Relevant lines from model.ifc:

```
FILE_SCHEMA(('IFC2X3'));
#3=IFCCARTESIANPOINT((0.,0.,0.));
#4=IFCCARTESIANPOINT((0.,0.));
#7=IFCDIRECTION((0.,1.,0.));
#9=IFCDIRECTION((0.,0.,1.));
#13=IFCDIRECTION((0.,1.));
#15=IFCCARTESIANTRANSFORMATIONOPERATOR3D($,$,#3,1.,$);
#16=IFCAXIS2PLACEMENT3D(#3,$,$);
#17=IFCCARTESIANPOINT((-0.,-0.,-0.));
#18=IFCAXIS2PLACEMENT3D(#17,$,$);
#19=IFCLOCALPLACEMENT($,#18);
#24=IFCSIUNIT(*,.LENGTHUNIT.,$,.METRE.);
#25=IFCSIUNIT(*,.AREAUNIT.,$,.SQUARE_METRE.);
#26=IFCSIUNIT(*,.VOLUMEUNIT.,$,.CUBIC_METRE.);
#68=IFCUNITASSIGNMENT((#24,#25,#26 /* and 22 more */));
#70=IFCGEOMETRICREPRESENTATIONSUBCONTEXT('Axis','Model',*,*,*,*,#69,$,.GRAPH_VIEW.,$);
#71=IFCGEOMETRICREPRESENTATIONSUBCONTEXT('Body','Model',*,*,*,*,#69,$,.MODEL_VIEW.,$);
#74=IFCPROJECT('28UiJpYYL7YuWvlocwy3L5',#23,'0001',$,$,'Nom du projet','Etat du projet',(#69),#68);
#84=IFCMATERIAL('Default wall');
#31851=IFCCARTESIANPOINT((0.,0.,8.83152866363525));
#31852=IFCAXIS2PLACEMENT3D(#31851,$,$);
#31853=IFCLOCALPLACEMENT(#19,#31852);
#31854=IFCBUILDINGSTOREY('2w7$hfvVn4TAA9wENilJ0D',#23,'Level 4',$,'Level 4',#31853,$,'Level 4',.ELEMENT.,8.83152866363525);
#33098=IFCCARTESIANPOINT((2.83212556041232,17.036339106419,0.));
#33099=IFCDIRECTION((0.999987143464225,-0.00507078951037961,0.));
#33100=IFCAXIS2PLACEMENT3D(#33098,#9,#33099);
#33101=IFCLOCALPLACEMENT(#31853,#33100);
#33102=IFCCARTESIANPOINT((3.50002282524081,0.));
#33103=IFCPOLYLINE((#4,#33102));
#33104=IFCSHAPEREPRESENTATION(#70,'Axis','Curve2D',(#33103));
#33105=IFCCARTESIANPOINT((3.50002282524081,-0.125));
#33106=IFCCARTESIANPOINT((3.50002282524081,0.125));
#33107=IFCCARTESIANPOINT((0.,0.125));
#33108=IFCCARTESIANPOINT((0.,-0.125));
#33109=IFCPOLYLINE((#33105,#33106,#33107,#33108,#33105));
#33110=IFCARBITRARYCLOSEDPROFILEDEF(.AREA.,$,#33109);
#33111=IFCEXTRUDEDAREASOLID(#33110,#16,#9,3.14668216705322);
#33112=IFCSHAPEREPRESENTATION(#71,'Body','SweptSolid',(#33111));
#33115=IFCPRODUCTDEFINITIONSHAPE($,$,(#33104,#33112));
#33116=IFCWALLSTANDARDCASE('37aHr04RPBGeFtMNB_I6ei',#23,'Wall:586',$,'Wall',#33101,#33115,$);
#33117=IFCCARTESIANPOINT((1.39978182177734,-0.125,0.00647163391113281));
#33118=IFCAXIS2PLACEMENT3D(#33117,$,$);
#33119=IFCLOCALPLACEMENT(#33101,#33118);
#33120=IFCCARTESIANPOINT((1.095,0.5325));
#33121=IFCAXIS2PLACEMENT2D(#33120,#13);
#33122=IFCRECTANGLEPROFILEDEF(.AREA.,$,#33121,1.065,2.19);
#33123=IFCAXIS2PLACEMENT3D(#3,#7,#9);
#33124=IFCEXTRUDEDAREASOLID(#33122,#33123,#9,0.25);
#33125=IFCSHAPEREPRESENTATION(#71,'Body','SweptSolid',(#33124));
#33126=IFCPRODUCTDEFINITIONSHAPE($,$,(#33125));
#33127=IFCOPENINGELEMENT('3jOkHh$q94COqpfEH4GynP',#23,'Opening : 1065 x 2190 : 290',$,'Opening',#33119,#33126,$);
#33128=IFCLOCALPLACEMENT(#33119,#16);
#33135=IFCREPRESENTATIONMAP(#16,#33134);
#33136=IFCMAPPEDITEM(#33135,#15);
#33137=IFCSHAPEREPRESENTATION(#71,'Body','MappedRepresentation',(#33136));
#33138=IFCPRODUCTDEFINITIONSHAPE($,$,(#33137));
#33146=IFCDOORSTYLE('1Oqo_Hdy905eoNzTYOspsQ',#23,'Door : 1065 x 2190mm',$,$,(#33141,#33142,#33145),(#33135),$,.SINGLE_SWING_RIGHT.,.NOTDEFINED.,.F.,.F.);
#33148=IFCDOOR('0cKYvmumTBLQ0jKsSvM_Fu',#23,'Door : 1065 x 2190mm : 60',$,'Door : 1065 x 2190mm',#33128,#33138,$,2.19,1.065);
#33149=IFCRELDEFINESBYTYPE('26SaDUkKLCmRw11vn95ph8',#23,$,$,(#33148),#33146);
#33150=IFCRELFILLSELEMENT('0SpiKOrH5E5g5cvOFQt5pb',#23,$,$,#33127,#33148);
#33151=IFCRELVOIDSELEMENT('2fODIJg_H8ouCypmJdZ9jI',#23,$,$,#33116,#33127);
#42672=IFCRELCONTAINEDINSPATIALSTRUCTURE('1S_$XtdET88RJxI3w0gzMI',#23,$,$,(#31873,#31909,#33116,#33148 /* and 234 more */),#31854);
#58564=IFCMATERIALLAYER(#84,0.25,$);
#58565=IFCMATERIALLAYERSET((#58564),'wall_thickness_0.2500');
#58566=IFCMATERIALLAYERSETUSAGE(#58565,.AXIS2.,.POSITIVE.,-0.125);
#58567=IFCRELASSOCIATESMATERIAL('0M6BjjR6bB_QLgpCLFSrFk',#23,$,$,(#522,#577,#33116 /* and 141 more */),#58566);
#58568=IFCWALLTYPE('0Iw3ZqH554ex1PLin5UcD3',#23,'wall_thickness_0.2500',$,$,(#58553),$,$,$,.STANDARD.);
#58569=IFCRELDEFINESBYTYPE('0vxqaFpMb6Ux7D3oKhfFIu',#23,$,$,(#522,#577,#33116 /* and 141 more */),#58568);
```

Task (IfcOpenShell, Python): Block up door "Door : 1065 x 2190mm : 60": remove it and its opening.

```python
import ifcopenshell
import ifcopenshell.api.feature
import ifcopenshell.api.root
import ifcopenshell.geom
import ifcopenshell.util.shape

model = ifcopenshell.open("model.ifc")
settings = ifcopenshell.geom.settings()


def volume(element):
    """Net volume in cubic metres, openings subtracted."""
    shape = ifcopenshell.geom.create_shape(settings, element)
    return ifcopenshell.util.shape.get_volume(shape.geometry)


door = model.by_id(33148)
opening = door.FillsVoids[0].RelatingOpeningElement
wall = opening.VoidsElements[0].RelatingBuildingElement
before = volume(wall)

ifcopenshell.api.root.remove_product(model, product=door)
ifcopenshell.api.feature.remove_feature(model, feature=opening)

after = volume(wall)

print(f"wall volume {before:.3f} -> {after:.3f} m3")

model.write("model_v2.ifc")
```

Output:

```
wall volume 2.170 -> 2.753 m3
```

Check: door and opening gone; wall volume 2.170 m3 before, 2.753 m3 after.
